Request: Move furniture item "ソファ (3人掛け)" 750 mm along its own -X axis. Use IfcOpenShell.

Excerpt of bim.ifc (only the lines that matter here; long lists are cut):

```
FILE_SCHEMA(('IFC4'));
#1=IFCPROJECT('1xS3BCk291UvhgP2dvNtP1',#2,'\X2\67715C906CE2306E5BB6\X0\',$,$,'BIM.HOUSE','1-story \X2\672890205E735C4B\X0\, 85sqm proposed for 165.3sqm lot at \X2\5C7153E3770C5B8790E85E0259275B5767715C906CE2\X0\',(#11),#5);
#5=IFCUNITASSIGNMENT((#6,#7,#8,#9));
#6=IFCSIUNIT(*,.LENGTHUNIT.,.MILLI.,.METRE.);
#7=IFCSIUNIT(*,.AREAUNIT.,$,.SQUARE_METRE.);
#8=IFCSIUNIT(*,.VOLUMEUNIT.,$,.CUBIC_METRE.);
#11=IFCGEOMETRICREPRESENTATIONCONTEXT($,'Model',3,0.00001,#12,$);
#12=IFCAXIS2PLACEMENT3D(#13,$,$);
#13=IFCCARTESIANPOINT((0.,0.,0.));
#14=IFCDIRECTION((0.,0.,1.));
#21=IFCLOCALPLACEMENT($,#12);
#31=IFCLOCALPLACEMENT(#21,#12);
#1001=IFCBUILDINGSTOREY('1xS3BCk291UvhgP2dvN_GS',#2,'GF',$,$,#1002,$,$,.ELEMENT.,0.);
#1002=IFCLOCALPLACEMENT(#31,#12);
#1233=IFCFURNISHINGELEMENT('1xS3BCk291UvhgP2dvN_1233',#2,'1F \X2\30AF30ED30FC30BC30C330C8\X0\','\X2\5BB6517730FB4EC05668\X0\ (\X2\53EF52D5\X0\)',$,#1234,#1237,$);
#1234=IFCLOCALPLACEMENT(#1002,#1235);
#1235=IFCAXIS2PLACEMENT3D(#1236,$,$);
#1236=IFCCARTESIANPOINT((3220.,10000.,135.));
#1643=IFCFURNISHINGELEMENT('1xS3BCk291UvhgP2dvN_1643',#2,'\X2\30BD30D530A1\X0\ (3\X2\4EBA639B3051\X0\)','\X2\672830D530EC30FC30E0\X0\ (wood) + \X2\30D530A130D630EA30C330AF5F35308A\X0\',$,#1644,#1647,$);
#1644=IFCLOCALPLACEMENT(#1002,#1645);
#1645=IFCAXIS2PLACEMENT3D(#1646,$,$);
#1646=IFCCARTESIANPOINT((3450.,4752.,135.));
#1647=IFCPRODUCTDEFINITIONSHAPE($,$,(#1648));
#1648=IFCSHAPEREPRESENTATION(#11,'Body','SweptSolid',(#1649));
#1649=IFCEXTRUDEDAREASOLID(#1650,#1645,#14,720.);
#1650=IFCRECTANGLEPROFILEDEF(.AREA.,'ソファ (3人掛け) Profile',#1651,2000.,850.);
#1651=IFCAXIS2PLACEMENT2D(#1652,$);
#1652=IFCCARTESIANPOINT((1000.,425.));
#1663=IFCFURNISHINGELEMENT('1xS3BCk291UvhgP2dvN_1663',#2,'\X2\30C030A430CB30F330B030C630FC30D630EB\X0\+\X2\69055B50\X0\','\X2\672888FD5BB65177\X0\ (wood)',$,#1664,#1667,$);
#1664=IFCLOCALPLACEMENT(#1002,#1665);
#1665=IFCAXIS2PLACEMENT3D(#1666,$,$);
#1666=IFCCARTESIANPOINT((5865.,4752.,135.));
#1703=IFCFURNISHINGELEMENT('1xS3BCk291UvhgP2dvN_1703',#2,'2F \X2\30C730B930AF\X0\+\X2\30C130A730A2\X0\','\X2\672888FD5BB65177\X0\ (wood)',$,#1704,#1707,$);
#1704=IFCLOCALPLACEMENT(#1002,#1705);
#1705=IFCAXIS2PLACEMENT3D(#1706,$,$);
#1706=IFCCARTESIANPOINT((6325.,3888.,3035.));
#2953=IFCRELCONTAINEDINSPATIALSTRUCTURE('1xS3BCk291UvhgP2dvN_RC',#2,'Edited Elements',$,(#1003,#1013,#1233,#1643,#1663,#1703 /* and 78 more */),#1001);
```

```python
import ifcopenshell
import ifcopenshell.api.geometry
import ifcopenshell.util.placement
import ifcopenshell.util.unit

model = ifcopenshell.open("bim.ifc")
unit_scale = ifcopenshell.util.unit.calculate_unit_scale(model)

item = model.by_id(1643)
matrix = ifcopenshell.util.placement.get_local_placement(item.ObjectPlacement)
matrix[:3, 3] -= matrix[:3, 0] * 0.75 / unit_scale
ifcopenshell.api.geometry.edit_object_placement(model, product=item, matrix=matrix, is_si=False)

print(ifcopenshell.util.placement.get_local_placement(item.ObjectPlacement).round(3) + 0.0)

model.write("bim_v2.ifc")
```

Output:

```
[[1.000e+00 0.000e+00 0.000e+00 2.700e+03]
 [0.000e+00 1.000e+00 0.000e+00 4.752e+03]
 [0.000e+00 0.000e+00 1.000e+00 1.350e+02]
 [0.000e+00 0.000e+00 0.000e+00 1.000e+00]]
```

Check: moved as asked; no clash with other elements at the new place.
